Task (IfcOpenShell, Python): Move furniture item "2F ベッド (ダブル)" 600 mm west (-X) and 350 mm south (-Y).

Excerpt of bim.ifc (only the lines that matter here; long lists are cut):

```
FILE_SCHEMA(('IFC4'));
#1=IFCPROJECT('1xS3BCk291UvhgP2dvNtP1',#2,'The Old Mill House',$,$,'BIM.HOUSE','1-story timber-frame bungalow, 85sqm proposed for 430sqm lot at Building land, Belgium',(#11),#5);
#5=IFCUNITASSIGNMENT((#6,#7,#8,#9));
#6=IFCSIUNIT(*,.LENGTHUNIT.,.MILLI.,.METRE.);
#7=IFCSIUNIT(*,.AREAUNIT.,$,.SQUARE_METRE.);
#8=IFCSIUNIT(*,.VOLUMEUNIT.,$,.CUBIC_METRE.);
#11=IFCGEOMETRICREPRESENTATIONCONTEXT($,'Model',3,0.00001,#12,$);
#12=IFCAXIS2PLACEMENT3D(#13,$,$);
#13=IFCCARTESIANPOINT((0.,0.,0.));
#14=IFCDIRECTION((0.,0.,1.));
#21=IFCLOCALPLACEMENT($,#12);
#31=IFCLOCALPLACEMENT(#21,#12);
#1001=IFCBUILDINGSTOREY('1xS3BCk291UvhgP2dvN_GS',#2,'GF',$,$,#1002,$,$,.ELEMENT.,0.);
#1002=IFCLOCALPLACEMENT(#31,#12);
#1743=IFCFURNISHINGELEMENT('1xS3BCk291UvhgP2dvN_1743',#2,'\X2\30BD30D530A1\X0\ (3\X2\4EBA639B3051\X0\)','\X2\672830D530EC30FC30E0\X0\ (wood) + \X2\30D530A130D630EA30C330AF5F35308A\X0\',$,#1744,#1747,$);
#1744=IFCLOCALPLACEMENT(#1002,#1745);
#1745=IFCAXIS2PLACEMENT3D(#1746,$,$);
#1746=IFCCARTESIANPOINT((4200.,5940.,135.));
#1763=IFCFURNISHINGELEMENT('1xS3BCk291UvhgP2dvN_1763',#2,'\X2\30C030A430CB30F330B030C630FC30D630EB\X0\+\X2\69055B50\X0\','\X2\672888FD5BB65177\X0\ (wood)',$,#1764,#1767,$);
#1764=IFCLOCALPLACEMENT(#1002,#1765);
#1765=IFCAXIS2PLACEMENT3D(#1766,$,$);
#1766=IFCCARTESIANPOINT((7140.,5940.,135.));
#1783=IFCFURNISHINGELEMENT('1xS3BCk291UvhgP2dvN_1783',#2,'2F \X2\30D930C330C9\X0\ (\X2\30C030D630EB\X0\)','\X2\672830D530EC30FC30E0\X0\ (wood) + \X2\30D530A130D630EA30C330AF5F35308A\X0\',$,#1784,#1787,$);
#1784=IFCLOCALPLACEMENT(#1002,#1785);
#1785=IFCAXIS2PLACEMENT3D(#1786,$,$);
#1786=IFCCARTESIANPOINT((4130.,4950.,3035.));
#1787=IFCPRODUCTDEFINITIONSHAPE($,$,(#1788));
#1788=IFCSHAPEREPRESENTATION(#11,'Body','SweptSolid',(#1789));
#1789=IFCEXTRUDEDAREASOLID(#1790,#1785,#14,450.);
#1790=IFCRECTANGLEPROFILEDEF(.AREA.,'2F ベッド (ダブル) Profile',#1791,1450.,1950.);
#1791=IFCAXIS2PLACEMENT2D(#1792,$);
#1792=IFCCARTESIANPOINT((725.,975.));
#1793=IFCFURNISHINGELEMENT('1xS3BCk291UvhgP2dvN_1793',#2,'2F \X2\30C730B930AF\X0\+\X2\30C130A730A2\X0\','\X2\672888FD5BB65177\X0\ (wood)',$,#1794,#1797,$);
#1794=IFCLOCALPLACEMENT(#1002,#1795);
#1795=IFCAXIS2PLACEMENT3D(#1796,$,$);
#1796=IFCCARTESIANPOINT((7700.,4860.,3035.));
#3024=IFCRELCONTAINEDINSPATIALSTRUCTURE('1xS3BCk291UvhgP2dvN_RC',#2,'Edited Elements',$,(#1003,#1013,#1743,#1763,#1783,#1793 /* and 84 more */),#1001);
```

```python
import ifcopenshell
import ifcopenshell.api.geometry
import ifcopenshell.util.placement

model = ifcopenshell.open("bim.ifc")

item = model.by_id(1783)
matrix = ifcopenshell.util.placement.get_local_placement(item.ObjectPlacement)
matrix[0, 3] -= 600.0
matrix[1, 3] -= 350.0
ifcopenshell.api.geometry.edit_object_placement(model, product=item, matrix=matrix, is_si=False)

print(ifcopenshell.util.placement.get_local_placement(item.ObjectPlacement).round(3) + 0.0)

model.write("bim-out.ifc")
```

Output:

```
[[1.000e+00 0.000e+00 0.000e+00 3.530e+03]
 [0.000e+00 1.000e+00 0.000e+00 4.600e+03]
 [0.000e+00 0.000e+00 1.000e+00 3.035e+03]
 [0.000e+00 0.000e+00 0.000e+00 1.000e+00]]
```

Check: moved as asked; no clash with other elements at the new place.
